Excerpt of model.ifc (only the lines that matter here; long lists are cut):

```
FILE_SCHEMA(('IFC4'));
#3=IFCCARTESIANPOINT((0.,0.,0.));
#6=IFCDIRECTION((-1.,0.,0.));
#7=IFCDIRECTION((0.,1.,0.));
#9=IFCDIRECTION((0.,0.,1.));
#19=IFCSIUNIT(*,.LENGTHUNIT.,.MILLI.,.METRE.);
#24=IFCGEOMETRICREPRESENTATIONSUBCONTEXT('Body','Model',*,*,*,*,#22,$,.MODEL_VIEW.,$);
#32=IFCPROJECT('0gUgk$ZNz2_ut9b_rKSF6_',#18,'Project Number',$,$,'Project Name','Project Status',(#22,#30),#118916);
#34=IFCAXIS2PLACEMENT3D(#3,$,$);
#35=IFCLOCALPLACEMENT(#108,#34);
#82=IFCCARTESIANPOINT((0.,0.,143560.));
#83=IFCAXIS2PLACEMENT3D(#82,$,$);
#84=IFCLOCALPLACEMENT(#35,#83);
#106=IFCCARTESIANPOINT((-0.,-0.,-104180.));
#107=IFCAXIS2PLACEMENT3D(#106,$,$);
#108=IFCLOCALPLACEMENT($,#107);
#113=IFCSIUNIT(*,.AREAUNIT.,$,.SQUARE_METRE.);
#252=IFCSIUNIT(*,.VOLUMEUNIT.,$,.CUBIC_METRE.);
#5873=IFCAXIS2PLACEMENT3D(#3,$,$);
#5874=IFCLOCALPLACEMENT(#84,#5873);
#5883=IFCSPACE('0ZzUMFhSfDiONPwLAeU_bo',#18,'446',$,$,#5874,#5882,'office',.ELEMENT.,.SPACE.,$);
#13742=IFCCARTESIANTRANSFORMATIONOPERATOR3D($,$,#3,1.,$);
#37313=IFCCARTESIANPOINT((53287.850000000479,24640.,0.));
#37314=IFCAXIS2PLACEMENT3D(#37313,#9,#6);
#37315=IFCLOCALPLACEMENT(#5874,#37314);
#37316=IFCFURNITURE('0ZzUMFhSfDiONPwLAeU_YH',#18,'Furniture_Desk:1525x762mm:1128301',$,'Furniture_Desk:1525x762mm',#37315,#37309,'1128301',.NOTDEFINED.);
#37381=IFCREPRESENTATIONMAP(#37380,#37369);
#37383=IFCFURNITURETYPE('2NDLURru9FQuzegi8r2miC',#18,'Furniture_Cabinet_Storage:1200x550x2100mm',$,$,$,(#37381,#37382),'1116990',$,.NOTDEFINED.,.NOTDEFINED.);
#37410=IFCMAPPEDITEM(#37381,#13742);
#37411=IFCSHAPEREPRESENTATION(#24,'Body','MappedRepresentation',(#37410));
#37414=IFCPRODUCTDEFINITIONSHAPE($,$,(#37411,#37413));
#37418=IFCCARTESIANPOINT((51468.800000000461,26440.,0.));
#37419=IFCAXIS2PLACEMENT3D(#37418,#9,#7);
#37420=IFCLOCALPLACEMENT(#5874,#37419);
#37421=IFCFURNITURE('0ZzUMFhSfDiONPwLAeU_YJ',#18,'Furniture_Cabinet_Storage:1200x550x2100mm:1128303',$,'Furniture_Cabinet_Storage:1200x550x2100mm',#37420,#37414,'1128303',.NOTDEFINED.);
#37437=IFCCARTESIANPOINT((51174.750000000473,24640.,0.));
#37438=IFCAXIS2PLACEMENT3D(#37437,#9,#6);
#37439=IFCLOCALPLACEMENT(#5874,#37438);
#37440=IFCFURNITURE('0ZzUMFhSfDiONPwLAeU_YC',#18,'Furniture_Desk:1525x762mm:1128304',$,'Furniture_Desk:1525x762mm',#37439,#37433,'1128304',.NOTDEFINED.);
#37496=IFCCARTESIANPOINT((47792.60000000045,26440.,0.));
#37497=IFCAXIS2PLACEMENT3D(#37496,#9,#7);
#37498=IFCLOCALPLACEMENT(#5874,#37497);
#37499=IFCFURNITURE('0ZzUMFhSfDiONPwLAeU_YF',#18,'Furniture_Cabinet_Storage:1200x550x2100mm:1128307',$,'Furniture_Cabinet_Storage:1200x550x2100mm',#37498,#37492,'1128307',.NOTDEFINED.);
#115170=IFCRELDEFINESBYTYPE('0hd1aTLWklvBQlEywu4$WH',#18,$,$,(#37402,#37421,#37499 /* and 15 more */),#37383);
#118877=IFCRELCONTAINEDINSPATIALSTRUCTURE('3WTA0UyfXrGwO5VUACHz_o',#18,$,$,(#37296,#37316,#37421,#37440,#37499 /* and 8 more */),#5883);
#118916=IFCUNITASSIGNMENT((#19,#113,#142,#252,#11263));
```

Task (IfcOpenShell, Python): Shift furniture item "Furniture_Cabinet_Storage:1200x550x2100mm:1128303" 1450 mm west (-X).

```python
import ifcopenshell
import ifcopenshell.api.geometry
import ifcopenshell.util.placement

model = ifcopenshell.open("model.ifc")

item = model.by_id(37421)
matrix = ifcopenshell.util.placement.get_local_placement(item.ObjectPlacement)
matrix[0, 3] -= 1450.0
ifcopenshell.api.geometry.edit_object_placement(model, product=item, matrix=matrix, is_si=False)

print(ifcopenshell.util.placement.get_local_placement(item.ObjectPlacement).round(3) + 0.0)

model.write("model-out.ifc")
```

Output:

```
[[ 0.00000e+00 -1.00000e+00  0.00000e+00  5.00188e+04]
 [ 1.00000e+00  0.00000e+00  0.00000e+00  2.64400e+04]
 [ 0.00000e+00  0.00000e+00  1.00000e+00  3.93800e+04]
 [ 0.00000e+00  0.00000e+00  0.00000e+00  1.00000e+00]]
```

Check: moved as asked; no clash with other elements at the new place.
